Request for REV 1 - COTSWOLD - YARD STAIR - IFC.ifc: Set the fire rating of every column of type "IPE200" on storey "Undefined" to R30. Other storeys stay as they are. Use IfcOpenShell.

First a look at what the model holds.

```python
import ifcopenshell
import ifcopenshell.util.element

model = ifcopenshell.open("REV 1 - COTSWOLD - YARD STAIR - IFC.ifc")
print(model.schema)
storey = next(s for s in model.by_type("IfcBuildingStorey") if s.Name == "Undefined")
columns = [e for e in ifcopenshell.util.element.get_decomposition(storey) if e.is_a("IfcColumn")]
seen = {}
for e in columns:
    element_type = ifcopenshell.util.element.get_type(e)
    key = (element_type.Name if element_type != e and element_type else None, ifcopenshell.util.element.get_pset(e, "Pset_ColumnCommon", "FireRating"))
    seen[key] = seen.get(key, 0) + 1
for (name, value), count in sorted(seen.items(), key=str):
    print(count, "x", name, "|", value)
```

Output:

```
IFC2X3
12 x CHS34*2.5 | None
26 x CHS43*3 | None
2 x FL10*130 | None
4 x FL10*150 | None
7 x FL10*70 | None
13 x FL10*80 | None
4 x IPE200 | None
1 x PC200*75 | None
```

```python
import ifcopenshell
import ifcopenshell.api.pset
import ifcopenshell.util.element

model = ifcopenshell.open("REV 1 - COTSWOLD - YARD STAIR - IFC.ifc")

storey = next(s for s in model.by_type("IfcBuildingStorey") if s.Name == "Undefined")
columns = [e for e in ifcopenshell.util.element.get_decomposition(storey) if e.is_a("IfcColumn")]

count = 0
for e in columns:
    element_type = ifcopenshell.util.element.get_type(e)
    if element_type in (None, e) or element_type.Name != "IPE200":
        continue
    # add_pset returns the element's existing set when there is one.
    pset = ifcopenshell.api.pset.add_pset(model, product=e, name="Pset_ColumnCommon")
    ifcopenshell.api.pset.edit_pset(model, pset=pset, properties={"FireRating": "R30"})
    count += 1

print(count, "columns updated")

model.write("REV 1 - COTSWOLD - YARD STAIR - IFC_v2.ifc")
```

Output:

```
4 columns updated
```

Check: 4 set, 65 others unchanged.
